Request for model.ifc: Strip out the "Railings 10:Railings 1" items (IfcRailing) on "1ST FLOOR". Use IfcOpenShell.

First a look at what the model holds.

```python
import ifcopenshell
import ifcopenshell.util.element

model = ifcopenshell.open("model.ifc")
print(model.schema)
storey = next(s for s in model.by_type("IfcBuildingStorey") if s.Name == "1ST FLOOR")
railings = [e for e in ifcopenshell.util.element.get_decomposition(storey) if e.is_a("IfcRailing")]
seen = {}
for e in railings:
    element_type = ifcopenshell.util.element.get_type(e)
    name = element_type.Name if element_type not in (None, e) else None
    seen[name] = seen.get(name, 0) + 1
for name, count in sorted(seen.items(), key=str):
    print(count, "x", name)
```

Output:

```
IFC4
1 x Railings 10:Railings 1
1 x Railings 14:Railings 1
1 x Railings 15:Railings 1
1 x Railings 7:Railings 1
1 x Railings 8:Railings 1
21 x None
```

```python
import ifcopenshell
import ifcopenshell.api.root
import ifcopenshell.util.element

model = ifcopenshell.open("model.ifc")

storey = next(s for s in model.by_type("IfcBuildingStorey") if s.Name == "1ST FLOOR")
railings = [e for e in ifcopenshell.util.element.get_decomposition(storey) if e.is_a("IfcRailing")]
targets = [e for e in railings if (t := ifcopenshell.util.element.get_type(e)) not in (None, e) and t.Name == "Railings 10:Railings 1"]

for e in targets:
    ifcopenshell.api.root.remove_product(model, product=e)
print(len(targets), "removed")

model.write("model-out.ifc")
```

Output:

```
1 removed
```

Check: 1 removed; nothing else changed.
